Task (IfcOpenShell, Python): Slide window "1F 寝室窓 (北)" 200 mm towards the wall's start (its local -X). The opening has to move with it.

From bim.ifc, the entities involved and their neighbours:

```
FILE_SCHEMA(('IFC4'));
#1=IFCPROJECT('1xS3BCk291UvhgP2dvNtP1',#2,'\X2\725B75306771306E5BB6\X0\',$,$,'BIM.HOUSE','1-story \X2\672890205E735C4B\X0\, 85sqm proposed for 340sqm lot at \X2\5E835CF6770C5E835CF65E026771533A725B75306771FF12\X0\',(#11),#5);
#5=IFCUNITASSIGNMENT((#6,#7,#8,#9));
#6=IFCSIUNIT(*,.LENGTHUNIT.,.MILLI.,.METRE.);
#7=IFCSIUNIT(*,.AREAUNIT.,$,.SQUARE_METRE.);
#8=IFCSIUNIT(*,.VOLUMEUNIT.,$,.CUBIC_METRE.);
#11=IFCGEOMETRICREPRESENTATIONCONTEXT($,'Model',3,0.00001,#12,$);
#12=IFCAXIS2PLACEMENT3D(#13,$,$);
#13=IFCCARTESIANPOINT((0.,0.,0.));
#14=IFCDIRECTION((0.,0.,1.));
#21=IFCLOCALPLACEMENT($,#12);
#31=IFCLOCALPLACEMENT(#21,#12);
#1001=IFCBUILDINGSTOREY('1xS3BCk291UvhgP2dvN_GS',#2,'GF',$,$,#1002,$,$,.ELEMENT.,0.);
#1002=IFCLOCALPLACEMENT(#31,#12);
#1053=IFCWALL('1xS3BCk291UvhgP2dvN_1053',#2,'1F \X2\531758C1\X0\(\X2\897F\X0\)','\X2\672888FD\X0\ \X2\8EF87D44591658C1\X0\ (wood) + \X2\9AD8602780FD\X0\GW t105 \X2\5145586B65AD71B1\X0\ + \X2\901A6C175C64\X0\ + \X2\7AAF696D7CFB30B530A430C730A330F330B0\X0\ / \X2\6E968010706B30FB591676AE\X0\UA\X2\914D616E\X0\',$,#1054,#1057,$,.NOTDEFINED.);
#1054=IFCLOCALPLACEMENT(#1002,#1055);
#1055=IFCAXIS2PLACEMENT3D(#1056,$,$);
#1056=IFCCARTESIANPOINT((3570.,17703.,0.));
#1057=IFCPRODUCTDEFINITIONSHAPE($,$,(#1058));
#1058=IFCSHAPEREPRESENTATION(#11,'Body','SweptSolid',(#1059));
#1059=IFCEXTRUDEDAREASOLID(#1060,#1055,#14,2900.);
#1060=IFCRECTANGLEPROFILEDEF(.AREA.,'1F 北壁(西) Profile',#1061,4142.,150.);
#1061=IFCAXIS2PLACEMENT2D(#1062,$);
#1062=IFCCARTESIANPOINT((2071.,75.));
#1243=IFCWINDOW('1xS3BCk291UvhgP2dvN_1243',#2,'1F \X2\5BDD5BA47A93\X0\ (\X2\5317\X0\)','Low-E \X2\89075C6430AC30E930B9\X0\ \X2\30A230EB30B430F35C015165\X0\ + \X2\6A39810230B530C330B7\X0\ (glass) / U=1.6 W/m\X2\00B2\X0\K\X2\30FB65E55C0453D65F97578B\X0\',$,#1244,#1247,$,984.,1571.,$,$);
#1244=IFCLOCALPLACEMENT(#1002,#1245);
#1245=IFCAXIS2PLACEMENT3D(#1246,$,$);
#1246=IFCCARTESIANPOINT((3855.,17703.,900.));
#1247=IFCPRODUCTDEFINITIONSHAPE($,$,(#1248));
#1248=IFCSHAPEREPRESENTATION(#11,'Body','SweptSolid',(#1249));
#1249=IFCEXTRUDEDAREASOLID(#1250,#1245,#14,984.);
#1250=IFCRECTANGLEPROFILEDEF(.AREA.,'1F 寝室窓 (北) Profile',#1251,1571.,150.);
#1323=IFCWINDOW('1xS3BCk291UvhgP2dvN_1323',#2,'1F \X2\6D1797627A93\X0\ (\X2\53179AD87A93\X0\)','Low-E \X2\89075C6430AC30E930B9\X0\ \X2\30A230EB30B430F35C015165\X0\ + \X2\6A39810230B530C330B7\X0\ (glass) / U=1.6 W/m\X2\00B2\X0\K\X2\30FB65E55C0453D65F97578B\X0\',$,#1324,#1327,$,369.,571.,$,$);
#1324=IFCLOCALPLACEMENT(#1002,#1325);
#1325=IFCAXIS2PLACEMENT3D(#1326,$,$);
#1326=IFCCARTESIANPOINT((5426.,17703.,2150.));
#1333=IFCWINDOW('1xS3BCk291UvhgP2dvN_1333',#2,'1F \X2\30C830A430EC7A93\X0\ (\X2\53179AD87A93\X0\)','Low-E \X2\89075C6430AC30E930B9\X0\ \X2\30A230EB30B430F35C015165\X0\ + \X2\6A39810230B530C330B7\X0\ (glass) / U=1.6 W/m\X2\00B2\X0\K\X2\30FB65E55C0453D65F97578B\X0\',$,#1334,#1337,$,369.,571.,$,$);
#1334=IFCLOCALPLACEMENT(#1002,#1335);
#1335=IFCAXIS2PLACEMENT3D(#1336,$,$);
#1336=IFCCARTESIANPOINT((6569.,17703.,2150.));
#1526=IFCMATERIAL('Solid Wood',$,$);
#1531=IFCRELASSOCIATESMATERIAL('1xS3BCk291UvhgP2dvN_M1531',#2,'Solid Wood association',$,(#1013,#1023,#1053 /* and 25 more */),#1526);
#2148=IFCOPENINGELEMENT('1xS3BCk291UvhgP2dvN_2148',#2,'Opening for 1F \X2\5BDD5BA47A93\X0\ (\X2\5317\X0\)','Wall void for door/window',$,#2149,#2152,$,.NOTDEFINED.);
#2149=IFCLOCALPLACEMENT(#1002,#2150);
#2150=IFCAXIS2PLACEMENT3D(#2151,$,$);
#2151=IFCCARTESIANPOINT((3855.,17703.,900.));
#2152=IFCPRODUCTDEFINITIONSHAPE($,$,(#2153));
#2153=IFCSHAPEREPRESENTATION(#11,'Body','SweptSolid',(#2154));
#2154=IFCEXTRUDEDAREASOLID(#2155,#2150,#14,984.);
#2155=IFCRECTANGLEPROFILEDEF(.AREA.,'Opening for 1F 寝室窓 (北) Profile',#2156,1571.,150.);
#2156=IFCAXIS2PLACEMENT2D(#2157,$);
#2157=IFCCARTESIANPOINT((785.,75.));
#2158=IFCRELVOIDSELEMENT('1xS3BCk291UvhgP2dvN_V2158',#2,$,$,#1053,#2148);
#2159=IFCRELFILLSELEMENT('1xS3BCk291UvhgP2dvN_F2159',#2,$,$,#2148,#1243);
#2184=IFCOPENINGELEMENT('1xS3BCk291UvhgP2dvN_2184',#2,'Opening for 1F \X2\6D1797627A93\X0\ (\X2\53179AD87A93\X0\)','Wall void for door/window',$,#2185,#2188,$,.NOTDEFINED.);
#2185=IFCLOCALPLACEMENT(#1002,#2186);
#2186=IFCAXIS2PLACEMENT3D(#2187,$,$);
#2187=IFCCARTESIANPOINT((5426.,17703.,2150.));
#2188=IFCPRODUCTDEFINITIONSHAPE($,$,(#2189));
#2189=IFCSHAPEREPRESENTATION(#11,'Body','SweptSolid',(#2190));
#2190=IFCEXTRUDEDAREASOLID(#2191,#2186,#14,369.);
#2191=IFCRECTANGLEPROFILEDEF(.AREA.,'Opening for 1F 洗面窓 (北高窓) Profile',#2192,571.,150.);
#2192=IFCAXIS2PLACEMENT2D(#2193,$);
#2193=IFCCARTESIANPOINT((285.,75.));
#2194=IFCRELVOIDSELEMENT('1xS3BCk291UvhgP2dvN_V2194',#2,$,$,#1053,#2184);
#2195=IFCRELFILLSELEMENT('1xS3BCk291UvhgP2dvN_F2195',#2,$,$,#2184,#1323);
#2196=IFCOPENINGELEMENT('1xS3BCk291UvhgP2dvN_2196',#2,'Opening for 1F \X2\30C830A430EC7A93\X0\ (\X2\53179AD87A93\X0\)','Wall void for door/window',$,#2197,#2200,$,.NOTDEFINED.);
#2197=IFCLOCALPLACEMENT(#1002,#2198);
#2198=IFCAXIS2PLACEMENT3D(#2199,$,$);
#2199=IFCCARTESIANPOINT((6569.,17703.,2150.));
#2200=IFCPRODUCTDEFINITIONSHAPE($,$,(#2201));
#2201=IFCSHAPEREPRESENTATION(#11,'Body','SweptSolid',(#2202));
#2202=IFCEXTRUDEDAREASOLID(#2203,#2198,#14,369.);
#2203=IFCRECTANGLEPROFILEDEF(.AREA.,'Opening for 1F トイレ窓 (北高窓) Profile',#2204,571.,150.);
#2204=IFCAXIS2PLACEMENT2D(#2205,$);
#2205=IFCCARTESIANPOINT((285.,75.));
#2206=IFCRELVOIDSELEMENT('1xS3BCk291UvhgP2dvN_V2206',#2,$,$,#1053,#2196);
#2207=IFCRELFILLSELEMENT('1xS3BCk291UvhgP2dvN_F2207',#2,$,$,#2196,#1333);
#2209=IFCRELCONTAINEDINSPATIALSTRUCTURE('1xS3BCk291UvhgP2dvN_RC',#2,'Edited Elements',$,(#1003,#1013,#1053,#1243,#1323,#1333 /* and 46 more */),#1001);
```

```python
import ifcopenshell
import ifcopenshell.api.geometry
import ifcopenshell.util.placement

model = ifcopenshell.open("bim.ifc")

window = model.by_guid("1xS3BCk291UvhgP2dvN_1243")
opening = window.FillsVoids[0].RelatingOpeningElement
wall = opening.VoidsElements[0].RelatingBuildingElement

wall_matrix = ifcopenshell.util.placement.get_local_placement(wall.ObjectPlacement)
shift = wall_matrix[:3, 0] * -200.0
before = ifcopenshell.util.placement.get_local_placement(window.ObjectPlacement)[:3, 3].copy()

# The window is not placed relative to its opening, so move both.
for product in (opening, window):
    matrix = ifcopenshell.util.placement.get_local_placement(product.ObjectPlacement)
    matrix[:3, 3] += shift
    ifcopenshell.api.geometry.edit_object_placement(model, product=product, matrix=matrix, is_si=False)

after = ifcopenshell.util.placement.get_local_placement(window.ObjectPlacement)[:3, 3]
print("window moved by", (after - before).round(3) + 0.0)

model.write("bim_v2.ifc")
```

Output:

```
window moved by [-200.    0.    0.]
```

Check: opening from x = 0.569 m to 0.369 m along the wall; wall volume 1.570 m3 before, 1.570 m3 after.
